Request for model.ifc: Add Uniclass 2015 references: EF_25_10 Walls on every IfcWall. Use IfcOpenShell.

First a look at what the model holds.

```python
import ifcopenshell

model = ifcopenshell.open("model.ifc")
print(model.schema)
print("classifications:", [c.Name for c in model.by_type("IfcClassification")])
for ifc_class in ("IfcDoor", "IfcRoof", "IfcStair", "IfcWall", "IfcWindow"):
    print(ifc_class, len(model.by_type(ifc_class)))
```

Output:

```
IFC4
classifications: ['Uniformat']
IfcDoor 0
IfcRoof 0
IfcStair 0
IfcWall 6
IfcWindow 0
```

```python
import ifcopenshell
import ifcopenshell.api.classification

model = ifcopenshell.open("model.ifc")

system = ifcopenshell.api.classification.add_classification(model, classification="Uniclass 2015")

codes = {
    "IfcWall": ("EF_25_10", "Walls"),
}
for ifc_class, (code, name) in codes.items():
    products = model.by_type(ifc_class)
    ifcopenshell.api.classification.add_reference(
        model, products=products, classification=system, identification=code, name=name
    )
    print(code, len(products))

model.write("model_v2.ifc")
```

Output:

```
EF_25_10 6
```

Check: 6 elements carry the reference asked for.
